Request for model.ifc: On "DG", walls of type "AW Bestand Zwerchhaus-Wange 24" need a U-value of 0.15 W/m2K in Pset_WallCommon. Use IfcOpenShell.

First a look at what the model holds.

```python
import ifcopenshell
import ifcopenshell.util.element

model = ifcopenshell.open("model.ifc")
print(model.schema)
storey = next(s for s in model.by_type("IfcBuildingStorey") if s.Name == "DG")
walls = [e for e in ifcopenshell.util.element.get_decomposition(storey) if e.is_a("IfcWall")]
seen = {}
for e in walls:
    element_type = ifcopenshell.util.element.get_type(e)
    key = (element_type.Name if element_type != e and element_type else None, ifcopenshell.util.element.get_pset(e, "Pset_WallCommon", "ThermalTransmittance"))
    seen[key] = seen.get(key, 0) + 1
for (name, value), count in sorted(seen.items(), key=str):
    print(count, "x", name, "|", value)
```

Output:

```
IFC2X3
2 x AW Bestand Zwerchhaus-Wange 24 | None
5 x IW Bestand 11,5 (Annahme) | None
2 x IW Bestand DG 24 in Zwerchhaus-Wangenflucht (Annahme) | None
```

```python
import ifcopenshell
import ifcopenshell.api.pset
import ifcopenshell.util.element

model = ifcopenshell.open("model.ifc")

storey = next(s for s in model.by_type("IfcBuildingStorey") if s.Name == "DG")
walls = [e for e in ifcopenshell.util.element.get_decomposition(storey) if e.is_a("IfcWall")]

count = 0
for e in walls:
    element_type = ifcopenshell.util.element.get_type(e)
    if element_type in (None, e) or element_type.Name != "AW Bestand Zwerchhaus-Wange 24":
        continue
    # add_pset returns the element's existing set when there is one.
    pset = ifcopenshell.api.pset.add_pset(model, product=e, name="Pset_WallCommon")
    ifcopenshell.api.pset.edit_pset(model, pset=pset, properties={"ThermalTransmittance": 0.15})
    count += 1

print(count, "walls updated")

model.write("model_rev.ifc")
```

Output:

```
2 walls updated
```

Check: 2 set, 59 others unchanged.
